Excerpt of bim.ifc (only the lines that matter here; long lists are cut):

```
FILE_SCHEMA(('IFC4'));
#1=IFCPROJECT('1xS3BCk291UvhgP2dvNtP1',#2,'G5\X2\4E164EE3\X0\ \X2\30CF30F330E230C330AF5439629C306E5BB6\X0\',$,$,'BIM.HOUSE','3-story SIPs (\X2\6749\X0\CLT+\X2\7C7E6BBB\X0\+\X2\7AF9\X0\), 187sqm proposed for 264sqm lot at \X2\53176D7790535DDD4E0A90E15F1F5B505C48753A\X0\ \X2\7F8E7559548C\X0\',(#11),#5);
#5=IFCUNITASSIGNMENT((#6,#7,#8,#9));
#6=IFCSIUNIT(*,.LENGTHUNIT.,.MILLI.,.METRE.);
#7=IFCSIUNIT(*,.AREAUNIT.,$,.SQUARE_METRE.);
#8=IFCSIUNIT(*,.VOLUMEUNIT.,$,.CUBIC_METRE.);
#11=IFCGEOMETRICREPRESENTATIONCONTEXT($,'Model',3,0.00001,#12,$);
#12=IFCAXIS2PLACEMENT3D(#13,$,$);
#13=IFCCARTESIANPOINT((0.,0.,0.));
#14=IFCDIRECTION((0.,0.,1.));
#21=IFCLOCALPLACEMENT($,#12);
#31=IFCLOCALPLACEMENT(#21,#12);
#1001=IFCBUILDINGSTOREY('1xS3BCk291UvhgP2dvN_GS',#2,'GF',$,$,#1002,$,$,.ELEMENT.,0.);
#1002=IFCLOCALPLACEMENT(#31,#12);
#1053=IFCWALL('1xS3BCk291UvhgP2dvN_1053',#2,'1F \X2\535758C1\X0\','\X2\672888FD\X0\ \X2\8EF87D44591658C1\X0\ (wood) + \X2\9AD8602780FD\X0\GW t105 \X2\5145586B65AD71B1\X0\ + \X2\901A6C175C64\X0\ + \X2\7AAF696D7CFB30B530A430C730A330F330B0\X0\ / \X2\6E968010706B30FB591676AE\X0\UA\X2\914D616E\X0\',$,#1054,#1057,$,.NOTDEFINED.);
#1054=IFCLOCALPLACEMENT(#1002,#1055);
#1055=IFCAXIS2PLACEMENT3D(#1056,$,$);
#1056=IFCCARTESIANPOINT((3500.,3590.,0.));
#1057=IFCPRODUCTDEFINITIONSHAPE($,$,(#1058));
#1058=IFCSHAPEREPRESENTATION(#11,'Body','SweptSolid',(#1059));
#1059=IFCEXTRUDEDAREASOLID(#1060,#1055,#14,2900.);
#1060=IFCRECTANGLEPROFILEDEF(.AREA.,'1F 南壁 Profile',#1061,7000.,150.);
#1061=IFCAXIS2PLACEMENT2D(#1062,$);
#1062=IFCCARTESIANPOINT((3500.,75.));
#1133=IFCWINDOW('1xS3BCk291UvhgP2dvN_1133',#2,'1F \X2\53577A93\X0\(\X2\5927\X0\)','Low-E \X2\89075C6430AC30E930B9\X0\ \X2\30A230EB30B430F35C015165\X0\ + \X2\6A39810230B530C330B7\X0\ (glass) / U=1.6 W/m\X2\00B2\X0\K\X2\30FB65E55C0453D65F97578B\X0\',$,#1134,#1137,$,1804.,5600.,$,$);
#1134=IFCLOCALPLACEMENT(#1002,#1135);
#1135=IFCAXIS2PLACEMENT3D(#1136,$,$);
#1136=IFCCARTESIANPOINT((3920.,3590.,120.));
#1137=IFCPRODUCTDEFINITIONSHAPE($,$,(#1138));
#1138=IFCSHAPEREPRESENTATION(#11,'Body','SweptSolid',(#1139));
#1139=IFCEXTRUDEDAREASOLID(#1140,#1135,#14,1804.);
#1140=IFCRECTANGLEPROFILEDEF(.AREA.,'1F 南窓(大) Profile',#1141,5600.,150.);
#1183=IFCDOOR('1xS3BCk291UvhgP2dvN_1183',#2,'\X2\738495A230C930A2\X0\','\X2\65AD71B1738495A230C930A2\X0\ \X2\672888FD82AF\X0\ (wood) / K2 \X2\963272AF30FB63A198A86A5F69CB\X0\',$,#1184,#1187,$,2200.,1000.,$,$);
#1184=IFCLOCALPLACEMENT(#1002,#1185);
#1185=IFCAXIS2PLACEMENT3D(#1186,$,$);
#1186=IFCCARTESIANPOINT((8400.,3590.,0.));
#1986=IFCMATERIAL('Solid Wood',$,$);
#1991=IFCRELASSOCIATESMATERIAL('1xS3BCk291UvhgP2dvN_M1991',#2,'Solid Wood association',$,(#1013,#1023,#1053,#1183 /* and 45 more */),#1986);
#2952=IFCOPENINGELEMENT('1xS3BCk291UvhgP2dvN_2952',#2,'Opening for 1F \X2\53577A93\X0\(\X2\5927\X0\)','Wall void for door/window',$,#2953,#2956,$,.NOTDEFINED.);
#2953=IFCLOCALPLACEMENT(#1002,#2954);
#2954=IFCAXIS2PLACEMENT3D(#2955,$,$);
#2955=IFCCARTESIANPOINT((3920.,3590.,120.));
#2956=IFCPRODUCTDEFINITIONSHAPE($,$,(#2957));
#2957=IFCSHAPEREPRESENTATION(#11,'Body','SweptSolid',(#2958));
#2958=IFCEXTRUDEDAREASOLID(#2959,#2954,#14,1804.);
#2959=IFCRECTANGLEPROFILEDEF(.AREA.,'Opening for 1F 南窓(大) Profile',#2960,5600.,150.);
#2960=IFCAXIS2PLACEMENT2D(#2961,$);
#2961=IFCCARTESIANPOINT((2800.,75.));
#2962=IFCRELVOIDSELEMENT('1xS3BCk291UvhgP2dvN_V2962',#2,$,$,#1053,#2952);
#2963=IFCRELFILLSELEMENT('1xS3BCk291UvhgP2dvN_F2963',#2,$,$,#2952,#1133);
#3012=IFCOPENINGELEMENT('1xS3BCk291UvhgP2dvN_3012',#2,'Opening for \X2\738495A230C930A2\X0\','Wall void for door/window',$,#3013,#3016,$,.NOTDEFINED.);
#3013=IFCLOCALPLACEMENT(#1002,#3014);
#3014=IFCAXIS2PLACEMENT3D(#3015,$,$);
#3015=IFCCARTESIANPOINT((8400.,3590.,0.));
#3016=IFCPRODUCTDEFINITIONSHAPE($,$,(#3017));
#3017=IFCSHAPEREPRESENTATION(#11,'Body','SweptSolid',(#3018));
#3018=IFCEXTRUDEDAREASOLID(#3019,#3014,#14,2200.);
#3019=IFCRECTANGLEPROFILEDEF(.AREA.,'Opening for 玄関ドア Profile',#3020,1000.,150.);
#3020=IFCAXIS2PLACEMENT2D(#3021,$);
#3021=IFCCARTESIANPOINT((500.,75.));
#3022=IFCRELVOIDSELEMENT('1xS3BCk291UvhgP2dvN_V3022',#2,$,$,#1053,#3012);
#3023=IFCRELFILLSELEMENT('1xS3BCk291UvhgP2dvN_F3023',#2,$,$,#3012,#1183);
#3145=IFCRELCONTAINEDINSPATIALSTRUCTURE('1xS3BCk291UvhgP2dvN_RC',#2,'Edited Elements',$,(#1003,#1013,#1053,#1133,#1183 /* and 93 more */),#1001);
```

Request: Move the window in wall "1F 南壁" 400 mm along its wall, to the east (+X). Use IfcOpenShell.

```python
import ifcopenshell
import ifcopenshell.api.geometry
import ifcopenshell.util.placement
import ifcopenshell.util.unit

model = ifcopenshell.open("bim.ifc")
unit_scale = ifcopenshell.util.unit.calculate_unit_scale(model)

window = model.by_id(1133)
opening = window.FillsVoids[0].RelatingOpeningElement
wall = opening.VoidsElements[0].RelatingBuildingElement

wall_matrix = ifcopenshell.util.placement.get_local_placement(wall.ObjectPlacement)
shift = wall_matrix[:3, 0] * 0.4 / unit_scale
before = ifcopenshell.util.placement.get_local_placement(window.ObjectPlacement)[:3, 3].copy()

# The window is not placed relative to its opening, so move both.
for product in (opening, window):
    matrix = ifcopenshell.util.placement.get_local_placement(product.ObjectPlacement)
    matrix[:3, 3] += shift
    ifcopenshell.api.geometry.edit_object_placement(model, product=product, matrix=matrix, is_si=False)

after = ifcopenshell.util.placement.get_local_placement(window.ObjectPlacement)[:3, 3]
print("window moved by", (after - before).round(3) + 0.0)

model.write("bim_rev.ifc")
```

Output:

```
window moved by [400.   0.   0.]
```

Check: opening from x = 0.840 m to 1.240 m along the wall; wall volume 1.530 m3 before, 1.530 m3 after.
